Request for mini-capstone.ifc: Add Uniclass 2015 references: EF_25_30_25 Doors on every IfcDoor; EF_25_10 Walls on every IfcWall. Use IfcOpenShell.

First a look at what the model holds.

```python
import ifcopenshell

model = ifcopenshell.open("mini-capstone.ifc")
print(model.schema)
print("classifications:", [c.Name for c in model.by_type("IfcClassification")])
for ifc_class in ("IfcDoor", "IfcRoof", "IfcStair", "IfcWall", "IfcWindow"):
    print(ifc_class, len(model.by_type(ifc_class)))
```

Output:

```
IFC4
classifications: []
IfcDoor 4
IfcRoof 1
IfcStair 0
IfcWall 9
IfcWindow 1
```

```python
import ifcopenshell
import ifcopenshell.api.classification

model = ifcopenshell.open("mini-capstone.ifc")

system = ifcopenshell.api.classification.add_classification(model, classification="Uniclass 2015")

codes = {
    "IfcDoor": ("EF_25_30_25", "Doors"),
    "IfcWall": ("EF_25_10", "Walls"),
}
for ifc_class, (code, name) in codes.items():
    products = model.by_type(ifc_class)
    ifcopenshell.api.classification.add_reference(
        model, products=products, classification=system, identification=code, name=name
    )
    print(code, len(products))

model.write("mini-capstone_edited.ifc")
```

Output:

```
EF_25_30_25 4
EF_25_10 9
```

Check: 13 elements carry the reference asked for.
